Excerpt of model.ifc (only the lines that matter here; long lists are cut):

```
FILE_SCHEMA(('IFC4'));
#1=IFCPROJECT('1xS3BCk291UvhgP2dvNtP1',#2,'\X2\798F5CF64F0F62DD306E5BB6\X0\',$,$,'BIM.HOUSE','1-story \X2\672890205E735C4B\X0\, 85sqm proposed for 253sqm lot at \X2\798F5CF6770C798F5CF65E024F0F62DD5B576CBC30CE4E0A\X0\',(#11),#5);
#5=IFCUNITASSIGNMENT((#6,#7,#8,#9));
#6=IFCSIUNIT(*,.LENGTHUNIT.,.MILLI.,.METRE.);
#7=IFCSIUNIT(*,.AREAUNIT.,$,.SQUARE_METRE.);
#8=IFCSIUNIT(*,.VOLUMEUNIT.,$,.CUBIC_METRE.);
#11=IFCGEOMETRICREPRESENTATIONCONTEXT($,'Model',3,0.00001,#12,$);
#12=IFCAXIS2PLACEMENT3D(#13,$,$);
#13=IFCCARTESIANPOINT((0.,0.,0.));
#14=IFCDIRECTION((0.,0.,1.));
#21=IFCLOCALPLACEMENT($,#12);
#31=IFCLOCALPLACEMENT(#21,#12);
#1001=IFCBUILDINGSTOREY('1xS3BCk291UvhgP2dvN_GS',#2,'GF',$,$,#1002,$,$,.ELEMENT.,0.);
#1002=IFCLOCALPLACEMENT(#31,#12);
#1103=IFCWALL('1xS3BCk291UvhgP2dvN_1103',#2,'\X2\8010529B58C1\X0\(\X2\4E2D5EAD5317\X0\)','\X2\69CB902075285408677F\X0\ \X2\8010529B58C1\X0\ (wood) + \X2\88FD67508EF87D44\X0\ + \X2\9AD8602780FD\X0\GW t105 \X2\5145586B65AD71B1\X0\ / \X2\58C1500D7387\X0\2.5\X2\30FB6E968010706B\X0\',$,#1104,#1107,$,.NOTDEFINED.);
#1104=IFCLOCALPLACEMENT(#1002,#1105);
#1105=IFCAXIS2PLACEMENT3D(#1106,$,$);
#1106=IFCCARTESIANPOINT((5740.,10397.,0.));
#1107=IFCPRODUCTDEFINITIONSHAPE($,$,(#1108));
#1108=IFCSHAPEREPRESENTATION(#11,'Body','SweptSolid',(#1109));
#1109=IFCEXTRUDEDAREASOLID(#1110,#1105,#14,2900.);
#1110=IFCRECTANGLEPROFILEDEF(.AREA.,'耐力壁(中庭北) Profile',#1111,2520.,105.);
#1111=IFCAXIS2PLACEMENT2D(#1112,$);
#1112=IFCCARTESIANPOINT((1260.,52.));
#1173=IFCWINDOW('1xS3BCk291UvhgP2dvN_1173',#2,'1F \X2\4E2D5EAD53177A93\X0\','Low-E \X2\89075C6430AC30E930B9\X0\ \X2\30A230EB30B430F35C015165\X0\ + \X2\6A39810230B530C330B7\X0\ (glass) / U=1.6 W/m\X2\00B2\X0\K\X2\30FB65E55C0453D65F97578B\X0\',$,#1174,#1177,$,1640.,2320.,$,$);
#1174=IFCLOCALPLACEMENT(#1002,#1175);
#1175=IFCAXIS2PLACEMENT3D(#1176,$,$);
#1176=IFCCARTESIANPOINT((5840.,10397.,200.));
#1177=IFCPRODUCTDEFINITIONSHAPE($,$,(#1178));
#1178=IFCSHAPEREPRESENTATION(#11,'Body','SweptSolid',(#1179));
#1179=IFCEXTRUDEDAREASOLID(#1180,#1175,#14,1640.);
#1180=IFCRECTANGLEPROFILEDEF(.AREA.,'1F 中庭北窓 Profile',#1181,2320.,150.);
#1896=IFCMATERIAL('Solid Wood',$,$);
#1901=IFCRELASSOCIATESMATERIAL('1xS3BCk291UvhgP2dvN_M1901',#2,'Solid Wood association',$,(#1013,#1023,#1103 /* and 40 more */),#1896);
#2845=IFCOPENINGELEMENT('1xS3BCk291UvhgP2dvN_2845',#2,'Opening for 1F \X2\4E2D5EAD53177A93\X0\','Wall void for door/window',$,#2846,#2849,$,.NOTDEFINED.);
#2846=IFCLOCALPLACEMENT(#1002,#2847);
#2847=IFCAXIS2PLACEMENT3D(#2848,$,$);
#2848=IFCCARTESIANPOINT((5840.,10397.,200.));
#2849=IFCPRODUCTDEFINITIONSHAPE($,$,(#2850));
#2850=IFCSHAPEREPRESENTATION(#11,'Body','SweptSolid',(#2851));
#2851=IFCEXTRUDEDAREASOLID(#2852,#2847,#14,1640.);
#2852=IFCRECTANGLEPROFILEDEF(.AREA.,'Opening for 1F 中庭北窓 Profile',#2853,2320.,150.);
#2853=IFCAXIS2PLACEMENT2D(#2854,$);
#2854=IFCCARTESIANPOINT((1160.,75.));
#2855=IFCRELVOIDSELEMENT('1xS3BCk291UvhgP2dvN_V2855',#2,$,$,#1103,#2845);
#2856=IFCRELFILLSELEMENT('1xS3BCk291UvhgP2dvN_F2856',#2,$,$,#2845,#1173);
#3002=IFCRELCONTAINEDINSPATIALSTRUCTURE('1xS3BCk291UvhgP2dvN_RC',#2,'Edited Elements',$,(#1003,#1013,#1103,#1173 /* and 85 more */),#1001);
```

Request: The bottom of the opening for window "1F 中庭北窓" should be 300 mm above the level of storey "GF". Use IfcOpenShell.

```python
import numpy as np
import ifcopenshell
import ifcopenshell.api.geometry
import ifcopenshell.geom
import ifcopenshell.util.element
import ifcopenshell.util.placement
import ifcopenshell.util.shape
import ifcopenshell.util.unit

model = ifcopenshell.open("model.ifc")
unit_scale = ifcopenshell.util.unit.calculate_unit_scale(model)

window = model.by_guid("1xS3BCk291UvhgP2dvN_1173")
opening = window.FillsVoids[0].RelatingOpeningElement
storey = ifcopenshell.util.element.get_container(window, ifc_class="IfcBuildingStorey")
level = ifcopenshell.util.placement.get_local_placement(storey.ObjectPlacement)[2, 3]

# The opening's origin need not be at the sill, so measure its lowest point.
shape = ifcopenshell.geom.create_shape(ifcopenshell.geom.settings(), opening)
bottom = ifcopenshell.util.shape.get_shape_bottom_elevation(shape, shape.geometry) / unit_scale
dz = level + 0.3 / unit_scale - bottom

shift = np.array([0.0, 0.0, dz])
# The window is not placed relative to its opening, so move both.
for product in (opening, window):
    matrix = ifcopenshell.util.placement.get_local_placement(product.ObjectPlacement)
    matrix[:3, 3] += shift
    ifcopenshell.api.geometry.edit_object_placement(model, product=product, matrix=matrix, is_si=False)

print(f"moved by {dz * unit_scale:+.3f} m")

model.write("model-out.ifc")
```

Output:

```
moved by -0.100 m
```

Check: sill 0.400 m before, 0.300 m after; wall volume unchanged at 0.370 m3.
